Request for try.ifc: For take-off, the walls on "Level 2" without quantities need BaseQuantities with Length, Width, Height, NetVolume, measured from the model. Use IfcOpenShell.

First a look at what the model holds.

```python
import ifcopenshell
import ifcopenshell.util.element
import ifcopenshell.util.unit

model = ifcopenshell.open("try.ifc")
print(model.schema)
for unit_type in ("LENGTHUNIT", "AREAUNIT", "VOLUMEUNIT"):
    print(unit_type, ifcopenshell.util.unit.calculate_unit_scale(model, unit_type))
storey = next(s for s in model.by_type("IfcBuildingStorey") if s.Name == "Level 2")
walls = [e for e in ifcopenshell.util.element.get_decomposition(storey) if e.is_a("IfcWall")]
for e in sorted(walls, key=lambda e: e.id()):
    print(e.id(), e.is_a(), e.Name, list(ifcopenshell.util.element.get_psets(e, qtos_only=True)), sep=" | ")
```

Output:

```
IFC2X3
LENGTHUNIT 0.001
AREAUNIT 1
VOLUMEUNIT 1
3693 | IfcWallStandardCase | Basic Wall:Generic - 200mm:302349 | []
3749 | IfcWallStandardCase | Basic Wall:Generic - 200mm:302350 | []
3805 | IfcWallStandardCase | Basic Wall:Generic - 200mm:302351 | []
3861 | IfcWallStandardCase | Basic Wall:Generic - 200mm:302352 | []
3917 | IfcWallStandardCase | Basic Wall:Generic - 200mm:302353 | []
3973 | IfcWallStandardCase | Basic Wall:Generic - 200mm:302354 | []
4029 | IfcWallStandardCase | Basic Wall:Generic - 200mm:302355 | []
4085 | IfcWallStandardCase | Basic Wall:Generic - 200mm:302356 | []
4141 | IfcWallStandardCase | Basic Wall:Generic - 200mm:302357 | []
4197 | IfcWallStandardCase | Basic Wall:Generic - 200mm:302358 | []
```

```python
import ifcopenshell
import ifcopenshell.api.pset
import ifcopenshell.geom
import ifcopenshell.util.element
import ifcopenshell.util.shape
import ifcopenshell.util.unit

model = ifcopenshell.open("try.ifc")
unit_scale = ifcopenshell.util.unit.calculate_unit_scale(model)
volume_scale = ifcopenshell.util.unit.calculate_unit_scale(model, "VOLUMEUNIT")
settings = ifcopenshell.geom.settings()

storey = next(s for s in model.by_type("IfcBuildingStorey") if s.Name == "Level 2")
walls = [e for e in ifcopenshell.util.element.get_decomposition(storey) if e.is_a("IfcWall")]

for e in sorted(walls, key=lambda e: e.id()):
    if ifcopenshell.util.element.get_psets(e, qtos_only=True, should_inherit=False):
        continue
    # Geometry comes back in metres, in the element's own axes.
    shape = ifcopenshell.geom.create_shape(settings, e)
    values = {
        "Length": ifcopenshell.util.shape.get_x(shape.geometry) / unit_scale,
        "Width": ifcopenshell.util.shape.get_y(shape.geometry) / unit_scale,
        "Height": ifcopenshell.util.shape.get_z(shape.geometry) / unit_scale,
        "NetVolume": ifcopenshell.util.shape.get_volume(shape.geometry) / volume_scale,
    }
    qto = ifcopenshell.api.pset.add_qto(model, product=e, name="BaseQuantities")
    ifcopenshell.api.pset.edit_qto(model, qto=qto, properties=values)
    print(e.id(), {k: round(v, 3) for k, v in values.items()})

model.write("try-out.ifc")
```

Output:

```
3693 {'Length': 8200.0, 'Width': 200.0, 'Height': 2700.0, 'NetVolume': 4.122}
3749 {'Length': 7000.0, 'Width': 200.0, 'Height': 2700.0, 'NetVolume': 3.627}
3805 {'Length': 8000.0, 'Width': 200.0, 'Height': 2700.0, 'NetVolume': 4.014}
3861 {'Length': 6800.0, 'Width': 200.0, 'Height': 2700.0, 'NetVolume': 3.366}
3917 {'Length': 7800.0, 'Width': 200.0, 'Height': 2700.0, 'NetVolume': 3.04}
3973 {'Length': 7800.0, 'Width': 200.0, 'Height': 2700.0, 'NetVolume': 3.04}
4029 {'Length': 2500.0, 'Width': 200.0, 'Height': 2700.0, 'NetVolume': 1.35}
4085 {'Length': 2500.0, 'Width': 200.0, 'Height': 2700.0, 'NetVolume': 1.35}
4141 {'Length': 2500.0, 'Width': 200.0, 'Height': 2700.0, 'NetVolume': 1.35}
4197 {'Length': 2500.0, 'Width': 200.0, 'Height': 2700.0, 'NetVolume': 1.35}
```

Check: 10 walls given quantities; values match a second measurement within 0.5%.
